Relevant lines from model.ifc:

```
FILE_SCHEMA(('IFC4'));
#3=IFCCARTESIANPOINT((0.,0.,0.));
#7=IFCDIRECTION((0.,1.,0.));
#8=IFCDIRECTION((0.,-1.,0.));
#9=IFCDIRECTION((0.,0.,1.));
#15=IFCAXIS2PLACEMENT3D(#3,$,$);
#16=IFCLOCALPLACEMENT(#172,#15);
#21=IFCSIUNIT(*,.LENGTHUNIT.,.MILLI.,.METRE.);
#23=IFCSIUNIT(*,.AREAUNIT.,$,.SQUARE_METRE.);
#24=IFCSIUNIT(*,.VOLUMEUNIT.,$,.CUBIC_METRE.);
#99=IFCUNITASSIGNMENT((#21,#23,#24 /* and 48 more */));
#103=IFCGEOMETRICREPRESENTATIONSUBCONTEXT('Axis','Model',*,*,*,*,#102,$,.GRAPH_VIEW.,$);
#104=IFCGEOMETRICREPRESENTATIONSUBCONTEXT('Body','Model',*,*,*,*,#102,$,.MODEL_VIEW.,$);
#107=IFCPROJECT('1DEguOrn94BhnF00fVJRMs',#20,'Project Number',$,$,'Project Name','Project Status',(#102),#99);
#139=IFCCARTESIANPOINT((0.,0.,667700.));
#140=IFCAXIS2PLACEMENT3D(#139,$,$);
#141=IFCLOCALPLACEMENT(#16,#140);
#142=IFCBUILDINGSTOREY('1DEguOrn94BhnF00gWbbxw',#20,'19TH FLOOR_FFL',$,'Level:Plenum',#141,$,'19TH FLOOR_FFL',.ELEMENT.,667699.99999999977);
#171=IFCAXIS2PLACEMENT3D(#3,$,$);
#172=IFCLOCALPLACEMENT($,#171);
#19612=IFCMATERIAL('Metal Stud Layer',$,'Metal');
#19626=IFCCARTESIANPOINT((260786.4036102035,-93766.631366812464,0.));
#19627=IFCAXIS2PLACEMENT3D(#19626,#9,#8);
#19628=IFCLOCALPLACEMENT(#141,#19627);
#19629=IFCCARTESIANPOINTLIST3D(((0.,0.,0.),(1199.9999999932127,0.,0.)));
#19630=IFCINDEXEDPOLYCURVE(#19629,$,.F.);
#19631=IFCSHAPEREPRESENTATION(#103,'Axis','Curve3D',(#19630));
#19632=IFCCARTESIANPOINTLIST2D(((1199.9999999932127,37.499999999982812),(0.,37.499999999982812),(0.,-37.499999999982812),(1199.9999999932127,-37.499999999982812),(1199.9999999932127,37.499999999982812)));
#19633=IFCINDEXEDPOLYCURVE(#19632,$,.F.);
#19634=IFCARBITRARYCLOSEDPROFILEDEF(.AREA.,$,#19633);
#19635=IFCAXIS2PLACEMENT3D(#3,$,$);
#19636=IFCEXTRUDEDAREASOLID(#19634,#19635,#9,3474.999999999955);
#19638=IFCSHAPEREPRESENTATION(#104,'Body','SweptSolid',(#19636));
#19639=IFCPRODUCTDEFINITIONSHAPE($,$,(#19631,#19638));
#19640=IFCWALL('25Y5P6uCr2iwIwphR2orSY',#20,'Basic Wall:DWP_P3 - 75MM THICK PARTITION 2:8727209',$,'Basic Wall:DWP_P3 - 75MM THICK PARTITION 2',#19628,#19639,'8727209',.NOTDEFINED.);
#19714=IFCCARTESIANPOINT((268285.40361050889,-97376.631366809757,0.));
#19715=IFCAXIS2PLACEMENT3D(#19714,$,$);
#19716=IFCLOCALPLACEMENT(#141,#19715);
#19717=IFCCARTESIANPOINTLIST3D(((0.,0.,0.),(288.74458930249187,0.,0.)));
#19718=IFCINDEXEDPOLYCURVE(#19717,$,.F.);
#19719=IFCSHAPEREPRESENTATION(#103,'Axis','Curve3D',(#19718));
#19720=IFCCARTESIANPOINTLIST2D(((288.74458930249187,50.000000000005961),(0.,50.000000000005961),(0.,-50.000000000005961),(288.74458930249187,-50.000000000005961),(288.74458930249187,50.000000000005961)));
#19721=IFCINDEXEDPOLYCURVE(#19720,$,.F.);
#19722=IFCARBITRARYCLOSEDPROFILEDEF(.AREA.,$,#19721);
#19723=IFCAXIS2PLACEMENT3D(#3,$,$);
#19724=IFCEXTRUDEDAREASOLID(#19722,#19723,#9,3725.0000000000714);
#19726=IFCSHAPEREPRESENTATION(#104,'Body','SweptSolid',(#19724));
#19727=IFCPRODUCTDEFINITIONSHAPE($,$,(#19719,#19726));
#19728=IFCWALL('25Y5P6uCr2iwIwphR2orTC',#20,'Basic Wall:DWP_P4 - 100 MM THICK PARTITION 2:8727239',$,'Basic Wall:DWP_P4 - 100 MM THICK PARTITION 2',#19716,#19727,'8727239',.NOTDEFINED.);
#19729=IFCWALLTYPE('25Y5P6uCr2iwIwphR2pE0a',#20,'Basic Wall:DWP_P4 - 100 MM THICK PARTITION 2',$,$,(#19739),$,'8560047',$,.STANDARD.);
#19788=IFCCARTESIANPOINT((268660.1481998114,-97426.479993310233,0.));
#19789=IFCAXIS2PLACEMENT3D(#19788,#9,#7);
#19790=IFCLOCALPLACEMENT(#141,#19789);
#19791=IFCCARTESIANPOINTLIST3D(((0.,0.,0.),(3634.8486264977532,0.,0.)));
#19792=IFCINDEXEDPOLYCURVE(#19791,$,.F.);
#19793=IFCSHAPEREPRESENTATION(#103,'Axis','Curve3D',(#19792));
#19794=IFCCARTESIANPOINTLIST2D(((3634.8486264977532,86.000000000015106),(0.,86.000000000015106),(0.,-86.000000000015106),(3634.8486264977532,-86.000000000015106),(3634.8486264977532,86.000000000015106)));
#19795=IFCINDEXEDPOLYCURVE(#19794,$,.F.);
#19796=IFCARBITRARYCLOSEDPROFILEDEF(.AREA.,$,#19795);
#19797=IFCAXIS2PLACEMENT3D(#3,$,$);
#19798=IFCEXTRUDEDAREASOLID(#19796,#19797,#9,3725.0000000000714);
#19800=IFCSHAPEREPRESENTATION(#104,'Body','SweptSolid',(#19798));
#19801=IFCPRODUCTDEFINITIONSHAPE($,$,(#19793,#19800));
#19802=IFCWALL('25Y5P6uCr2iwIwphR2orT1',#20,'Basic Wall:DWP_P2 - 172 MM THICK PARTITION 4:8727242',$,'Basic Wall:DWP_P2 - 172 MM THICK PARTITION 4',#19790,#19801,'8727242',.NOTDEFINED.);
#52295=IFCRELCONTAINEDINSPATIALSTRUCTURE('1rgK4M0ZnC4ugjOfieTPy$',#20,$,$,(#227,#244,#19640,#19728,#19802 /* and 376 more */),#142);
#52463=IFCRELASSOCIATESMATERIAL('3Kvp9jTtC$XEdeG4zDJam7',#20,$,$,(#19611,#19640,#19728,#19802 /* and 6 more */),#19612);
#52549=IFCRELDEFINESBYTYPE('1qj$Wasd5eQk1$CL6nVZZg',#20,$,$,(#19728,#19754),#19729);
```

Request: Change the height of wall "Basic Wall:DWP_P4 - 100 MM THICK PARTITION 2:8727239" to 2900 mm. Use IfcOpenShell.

```python
import ifcopenshell
import ifcopenshell.geom
import ifcopenshell.util.representation
import ifcopenshell.util.shape

model = ifcopenshell.open("model.ifc")
settings = ifcopenshell.geom.settings()


def volume(element):
    """Net volume in cubic metres, openings subtracted."""
    shape = ifcopenshell.geom.create_shape(settings, element)
    return ifcopenshell.util.shape.get_volume(shape.geometry)


wall = model.by_guid("25Y5P6uCr2iwIwphR2orTC")
before = volume(wall)

body = ifcopenshell.util.representation.get_representation(wall, "Model", "Body")
solid = body.Items[0]
old_height = solid.Depth
solid.Depth = 2900.0
after = volume(wall)

print(f"height {old_height:g} -> {solid.Depth:g}, volume {before:.3f} -> {after:.3f} m3")

model.write("model-out.ifc")
```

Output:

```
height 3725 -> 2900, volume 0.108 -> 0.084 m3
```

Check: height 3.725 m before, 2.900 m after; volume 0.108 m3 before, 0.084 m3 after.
